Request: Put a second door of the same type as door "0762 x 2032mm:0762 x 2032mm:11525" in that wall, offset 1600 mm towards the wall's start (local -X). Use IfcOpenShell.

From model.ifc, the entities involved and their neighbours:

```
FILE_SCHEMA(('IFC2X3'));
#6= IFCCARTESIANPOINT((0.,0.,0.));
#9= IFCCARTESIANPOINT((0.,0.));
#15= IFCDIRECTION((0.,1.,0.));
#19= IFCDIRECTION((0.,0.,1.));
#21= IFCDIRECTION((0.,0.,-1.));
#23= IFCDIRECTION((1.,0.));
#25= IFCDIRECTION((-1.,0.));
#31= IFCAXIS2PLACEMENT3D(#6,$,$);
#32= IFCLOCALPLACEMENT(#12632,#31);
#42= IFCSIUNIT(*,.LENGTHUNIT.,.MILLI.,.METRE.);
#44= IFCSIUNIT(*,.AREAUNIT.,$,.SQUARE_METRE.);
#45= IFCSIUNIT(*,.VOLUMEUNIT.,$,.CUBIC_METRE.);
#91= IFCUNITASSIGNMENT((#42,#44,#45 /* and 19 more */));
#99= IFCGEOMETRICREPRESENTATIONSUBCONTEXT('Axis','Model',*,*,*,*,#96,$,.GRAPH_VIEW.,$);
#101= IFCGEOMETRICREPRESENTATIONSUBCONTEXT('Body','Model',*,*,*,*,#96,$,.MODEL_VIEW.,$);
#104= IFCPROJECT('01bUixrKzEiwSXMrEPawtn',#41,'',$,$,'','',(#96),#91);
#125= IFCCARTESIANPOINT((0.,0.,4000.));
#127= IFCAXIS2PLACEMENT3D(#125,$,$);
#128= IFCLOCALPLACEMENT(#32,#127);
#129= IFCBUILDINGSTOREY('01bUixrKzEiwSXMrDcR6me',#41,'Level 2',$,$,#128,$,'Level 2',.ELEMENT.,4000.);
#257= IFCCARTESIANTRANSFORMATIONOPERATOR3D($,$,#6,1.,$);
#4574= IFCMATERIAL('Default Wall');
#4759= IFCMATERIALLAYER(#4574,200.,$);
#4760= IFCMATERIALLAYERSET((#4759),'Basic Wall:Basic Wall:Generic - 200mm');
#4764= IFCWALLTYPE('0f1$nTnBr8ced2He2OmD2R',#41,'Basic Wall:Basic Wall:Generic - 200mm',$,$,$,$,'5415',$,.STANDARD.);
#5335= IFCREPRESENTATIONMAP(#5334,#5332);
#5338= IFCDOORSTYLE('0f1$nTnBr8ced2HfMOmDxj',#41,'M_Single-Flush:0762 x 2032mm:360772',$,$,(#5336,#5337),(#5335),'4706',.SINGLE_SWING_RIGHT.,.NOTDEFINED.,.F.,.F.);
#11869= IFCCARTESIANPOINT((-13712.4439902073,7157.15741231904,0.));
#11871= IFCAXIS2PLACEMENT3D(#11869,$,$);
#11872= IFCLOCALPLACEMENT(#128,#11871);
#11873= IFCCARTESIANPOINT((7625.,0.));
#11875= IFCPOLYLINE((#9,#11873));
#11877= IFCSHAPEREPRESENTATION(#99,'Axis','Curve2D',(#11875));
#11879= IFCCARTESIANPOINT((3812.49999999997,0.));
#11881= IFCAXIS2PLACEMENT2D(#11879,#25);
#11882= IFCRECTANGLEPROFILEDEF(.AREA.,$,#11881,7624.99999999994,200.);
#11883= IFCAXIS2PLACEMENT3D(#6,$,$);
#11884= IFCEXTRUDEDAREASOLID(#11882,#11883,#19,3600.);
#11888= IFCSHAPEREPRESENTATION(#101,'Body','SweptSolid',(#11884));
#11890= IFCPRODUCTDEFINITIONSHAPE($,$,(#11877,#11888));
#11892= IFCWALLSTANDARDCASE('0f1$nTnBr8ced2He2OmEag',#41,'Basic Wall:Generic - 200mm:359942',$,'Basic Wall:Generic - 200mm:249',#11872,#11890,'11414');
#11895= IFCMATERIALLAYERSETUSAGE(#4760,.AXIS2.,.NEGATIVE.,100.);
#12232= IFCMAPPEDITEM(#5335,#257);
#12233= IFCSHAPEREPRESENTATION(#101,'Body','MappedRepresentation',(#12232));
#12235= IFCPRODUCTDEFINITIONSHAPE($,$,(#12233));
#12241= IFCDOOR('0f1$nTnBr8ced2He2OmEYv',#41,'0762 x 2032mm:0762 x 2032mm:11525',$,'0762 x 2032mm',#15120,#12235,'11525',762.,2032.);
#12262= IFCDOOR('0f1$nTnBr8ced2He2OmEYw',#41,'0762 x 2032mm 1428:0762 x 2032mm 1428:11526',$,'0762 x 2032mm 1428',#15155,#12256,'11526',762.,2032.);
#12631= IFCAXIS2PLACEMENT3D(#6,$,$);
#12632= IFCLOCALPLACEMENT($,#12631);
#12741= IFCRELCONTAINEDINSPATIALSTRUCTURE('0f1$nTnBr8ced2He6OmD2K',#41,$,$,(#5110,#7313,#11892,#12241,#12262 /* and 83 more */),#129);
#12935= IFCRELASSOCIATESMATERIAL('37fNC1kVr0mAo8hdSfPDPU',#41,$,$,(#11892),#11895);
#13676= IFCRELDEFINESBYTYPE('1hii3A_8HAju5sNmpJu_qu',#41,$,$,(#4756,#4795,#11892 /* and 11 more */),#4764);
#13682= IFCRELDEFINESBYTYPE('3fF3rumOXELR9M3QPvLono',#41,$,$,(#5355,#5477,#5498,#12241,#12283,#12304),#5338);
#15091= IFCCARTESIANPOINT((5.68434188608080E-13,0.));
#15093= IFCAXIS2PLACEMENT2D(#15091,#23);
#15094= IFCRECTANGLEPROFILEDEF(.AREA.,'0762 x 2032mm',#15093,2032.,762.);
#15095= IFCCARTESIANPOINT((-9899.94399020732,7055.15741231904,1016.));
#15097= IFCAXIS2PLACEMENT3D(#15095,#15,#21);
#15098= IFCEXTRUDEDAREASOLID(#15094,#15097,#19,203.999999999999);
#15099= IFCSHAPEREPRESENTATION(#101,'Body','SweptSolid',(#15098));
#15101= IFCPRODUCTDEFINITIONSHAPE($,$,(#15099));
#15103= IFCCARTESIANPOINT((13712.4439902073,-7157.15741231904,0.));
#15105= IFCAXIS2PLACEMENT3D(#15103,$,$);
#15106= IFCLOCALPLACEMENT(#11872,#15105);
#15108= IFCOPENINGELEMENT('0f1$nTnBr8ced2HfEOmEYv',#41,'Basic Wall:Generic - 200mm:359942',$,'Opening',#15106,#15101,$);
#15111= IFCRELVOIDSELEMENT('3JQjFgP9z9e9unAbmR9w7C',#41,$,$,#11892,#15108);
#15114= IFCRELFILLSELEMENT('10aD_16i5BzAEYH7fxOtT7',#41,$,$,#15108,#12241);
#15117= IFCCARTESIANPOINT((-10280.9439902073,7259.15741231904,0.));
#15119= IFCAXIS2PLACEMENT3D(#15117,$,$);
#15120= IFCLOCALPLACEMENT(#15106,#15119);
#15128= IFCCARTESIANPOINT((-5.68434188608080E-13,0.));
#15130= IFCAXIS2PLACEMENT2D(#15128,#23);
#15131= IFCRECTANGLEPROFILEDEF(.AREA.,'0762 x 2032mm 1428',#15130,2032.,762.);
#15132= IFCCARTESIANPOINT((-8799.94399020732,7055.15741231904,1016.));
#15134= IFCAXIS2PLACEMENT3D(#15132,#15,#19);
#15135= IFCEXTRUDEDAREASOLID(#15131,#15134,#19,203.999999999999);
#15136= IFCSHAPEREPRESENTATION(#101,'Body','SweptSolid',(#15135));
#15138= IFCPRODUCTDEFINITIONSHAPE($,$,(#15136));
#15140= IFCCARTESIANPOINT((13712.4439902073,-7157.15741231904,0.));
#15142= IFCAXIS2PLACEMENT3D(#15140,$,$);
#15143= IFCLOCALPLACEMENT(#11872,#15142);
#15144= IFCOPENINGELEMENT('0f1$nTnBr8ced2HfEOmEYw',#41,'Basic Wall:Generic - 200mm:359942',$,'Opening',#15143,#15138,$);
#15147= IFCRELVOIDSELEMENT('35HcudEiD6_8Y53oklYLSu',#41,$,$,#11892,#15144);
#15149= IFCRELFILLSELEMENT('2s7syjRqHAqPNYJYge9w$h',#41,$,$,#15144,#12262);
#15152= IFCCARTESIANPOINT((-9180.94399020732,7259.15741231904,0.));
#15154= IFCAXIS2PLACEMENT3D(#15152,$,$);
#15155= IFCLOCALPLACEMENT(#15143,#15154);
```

```python
import ifcopenshell
import ifcopenshell.api.feature
import ifcopenshell.api.geometry
import ifcopenshell.api.root
import ifcopenshell.geom
import ifcopenshell.util.element
import ifcopenshell.util.placement
import ifcopenshell.util.shape
import ifcopenshell.util.unit

model = ifcopenshell.open("model.ifc")
unit_scale = ifcopenshell.util.unit.calculate_unit_scale(model)
settings = ifcopenshell.geom.settings()


def volume(element):
    """Net volume in cubic metres, openings subtracted."""
    shape = ifcopenshell.geom.create_shape(settings, element)
    return ifcopenshell.util.shape.get_volume(shape.geometry)


def reuse_history(source, copy):
    """copy_class also copies each property set's owner history, people and application; keep the originals."""
    for rel in copy.IsDefinedBy:
        if rel.is_a("IfcRelDefinesByProperties") and (history := rel.RelatingPropertyDefinition.OwnerHistory):
            rel.RelatingPropertyDefinition.OwnerHistory = source.OwnerHistory
            ifcopenshell.util.element.remove_deep2(model, history)


door = model.by_id(12241)
opening = door.FillsVoids[0].RelatingOpeningElement
wall = opening.VoidsElements[0].RelatingBuildingElement
before = volume(wall)
shift = ifcopenshell.util.placement.get_local_placement(wall.ObjectPlacement)[:3, 0] * -1.6 / unit_scale

# copy_class copies the void relationship, type, container and properties, but no geometry.
new_opening = ifcopenshell.api.root.copy_class(model, product=opening)
new_opening.Representation = ifcopenshell.util.element.copy_deep(
    model, opening.Representation, exclude=["IfcGeometricRepresentationContext", "IfcRepresentationMap"]
)
new_opening.Name = "Basic Wall:Generic - 200mm"
new_door = ifcopenshell.api.root.copy_class(model, product=door)
new_door.Representation = ifcopenshell.util.element.copy_deep(
    model, door.Representation, exclude=["IfcGeometricRepresentationContext", "IfcRepresentationMap"]
)
new_door.Name = "0762 x 2032mm:0762 x 2032mm"
new_door.Tag = None
reuse_history(door, new_door)
fills = ifcopenshell.api.feature.add_filling(model, opening=new_opening, element=new_door)
fills.OwnerHistory = new_door.OwnerHistory  # required in IFC2X3

for old, new in ((opening, new_opening), (door, new_door)):
    matrix = ifcopenshell.util.placement.get_local_placement(old.ObjectPlacement)
    matrix[:3, 3] += shift
    ifcopenshell.api.geometry.edit_object_placement(model, product=new, matrix=matrix, is_si=False)

after = volume(wall)

print(f"wall volume {before:.3f} -> {after:.3f} m3")

model.write("model_v2.ifc")
```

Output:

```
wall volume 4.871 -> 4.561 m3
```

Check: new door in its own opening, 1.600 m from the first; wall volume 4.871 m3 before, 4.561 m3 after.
